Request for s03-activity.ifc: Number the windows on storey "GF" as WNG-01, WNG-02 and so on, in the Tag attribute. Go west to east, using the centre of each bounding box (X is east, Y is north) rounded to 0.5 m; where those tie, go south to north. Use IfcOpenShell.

First a look at what the model holds.

```python
import ifcopenshell
import ifcopenshell.util.element
import ifcopenshell.util.placement

model = ifcopenshell.open("s03-activity.ifc")
print(model.schema)
storey = next(s for s in model.by_type("IfcBuildingStorey") if s.Name == "GF")
windows = [e for e in ifcopenshell.util.element.get_decomposition(storey) if e.is_a("IfcWindow")]
for e in sorted(windows, key=lambda e: e.id()):
    origin = ifcopenshell.util.placement.get_local_placement(e.ObjectPlacement)[:3, 3]
    print(e.id(), e.Tag, e.Name, origin.round(2) + 0.0, sep=" | ")
```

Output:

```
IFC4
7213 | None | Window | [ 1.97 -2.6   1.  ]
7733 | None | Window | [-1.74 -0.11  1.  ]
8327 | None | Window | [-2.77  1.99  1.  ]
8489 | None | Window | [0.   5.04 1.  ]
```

```python
import ifcopenshell
import ifcopenshell.geom
import ifcopenshell.util.element
import ifcopenshell.util.shape

model = ifcopenshell.open("s03-activity.ifc")
settings = ifcopenshell.geom.settings()
settings.set("use-world-coords", True)


def centre(element):
    shape = ifcopenshell.geom.create_shape(settings, element)
    return ifcopenshell.util.shape.get_bbox_centroid(shape.geometry)


storey = next(s for s in model.by_type("IfcBuildingStorey") if s.Name == "GF")
windows = [e for e in ifcopenshell.util.element.get_decomposition(storey) if e.is_a("IfcWindow")]

# Insertion points can sit at a corner or the storey origin, so sort by the geometry (in metres).
centres = {e: centre(e) for e in windows}
windows.sort(key=lambda e: (round(centres[e][0] / 0.5), centres[e][1]))

for i, e in enumerate(windows, start=1):
    number = f"WNG-{i:02d}"
    e.Tag = number
    print(e.id(), number)

model.write("s03-activity-out.ifc")
```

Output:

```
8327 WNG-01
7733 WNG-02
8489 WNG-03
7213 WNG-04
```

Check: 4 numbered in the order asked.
